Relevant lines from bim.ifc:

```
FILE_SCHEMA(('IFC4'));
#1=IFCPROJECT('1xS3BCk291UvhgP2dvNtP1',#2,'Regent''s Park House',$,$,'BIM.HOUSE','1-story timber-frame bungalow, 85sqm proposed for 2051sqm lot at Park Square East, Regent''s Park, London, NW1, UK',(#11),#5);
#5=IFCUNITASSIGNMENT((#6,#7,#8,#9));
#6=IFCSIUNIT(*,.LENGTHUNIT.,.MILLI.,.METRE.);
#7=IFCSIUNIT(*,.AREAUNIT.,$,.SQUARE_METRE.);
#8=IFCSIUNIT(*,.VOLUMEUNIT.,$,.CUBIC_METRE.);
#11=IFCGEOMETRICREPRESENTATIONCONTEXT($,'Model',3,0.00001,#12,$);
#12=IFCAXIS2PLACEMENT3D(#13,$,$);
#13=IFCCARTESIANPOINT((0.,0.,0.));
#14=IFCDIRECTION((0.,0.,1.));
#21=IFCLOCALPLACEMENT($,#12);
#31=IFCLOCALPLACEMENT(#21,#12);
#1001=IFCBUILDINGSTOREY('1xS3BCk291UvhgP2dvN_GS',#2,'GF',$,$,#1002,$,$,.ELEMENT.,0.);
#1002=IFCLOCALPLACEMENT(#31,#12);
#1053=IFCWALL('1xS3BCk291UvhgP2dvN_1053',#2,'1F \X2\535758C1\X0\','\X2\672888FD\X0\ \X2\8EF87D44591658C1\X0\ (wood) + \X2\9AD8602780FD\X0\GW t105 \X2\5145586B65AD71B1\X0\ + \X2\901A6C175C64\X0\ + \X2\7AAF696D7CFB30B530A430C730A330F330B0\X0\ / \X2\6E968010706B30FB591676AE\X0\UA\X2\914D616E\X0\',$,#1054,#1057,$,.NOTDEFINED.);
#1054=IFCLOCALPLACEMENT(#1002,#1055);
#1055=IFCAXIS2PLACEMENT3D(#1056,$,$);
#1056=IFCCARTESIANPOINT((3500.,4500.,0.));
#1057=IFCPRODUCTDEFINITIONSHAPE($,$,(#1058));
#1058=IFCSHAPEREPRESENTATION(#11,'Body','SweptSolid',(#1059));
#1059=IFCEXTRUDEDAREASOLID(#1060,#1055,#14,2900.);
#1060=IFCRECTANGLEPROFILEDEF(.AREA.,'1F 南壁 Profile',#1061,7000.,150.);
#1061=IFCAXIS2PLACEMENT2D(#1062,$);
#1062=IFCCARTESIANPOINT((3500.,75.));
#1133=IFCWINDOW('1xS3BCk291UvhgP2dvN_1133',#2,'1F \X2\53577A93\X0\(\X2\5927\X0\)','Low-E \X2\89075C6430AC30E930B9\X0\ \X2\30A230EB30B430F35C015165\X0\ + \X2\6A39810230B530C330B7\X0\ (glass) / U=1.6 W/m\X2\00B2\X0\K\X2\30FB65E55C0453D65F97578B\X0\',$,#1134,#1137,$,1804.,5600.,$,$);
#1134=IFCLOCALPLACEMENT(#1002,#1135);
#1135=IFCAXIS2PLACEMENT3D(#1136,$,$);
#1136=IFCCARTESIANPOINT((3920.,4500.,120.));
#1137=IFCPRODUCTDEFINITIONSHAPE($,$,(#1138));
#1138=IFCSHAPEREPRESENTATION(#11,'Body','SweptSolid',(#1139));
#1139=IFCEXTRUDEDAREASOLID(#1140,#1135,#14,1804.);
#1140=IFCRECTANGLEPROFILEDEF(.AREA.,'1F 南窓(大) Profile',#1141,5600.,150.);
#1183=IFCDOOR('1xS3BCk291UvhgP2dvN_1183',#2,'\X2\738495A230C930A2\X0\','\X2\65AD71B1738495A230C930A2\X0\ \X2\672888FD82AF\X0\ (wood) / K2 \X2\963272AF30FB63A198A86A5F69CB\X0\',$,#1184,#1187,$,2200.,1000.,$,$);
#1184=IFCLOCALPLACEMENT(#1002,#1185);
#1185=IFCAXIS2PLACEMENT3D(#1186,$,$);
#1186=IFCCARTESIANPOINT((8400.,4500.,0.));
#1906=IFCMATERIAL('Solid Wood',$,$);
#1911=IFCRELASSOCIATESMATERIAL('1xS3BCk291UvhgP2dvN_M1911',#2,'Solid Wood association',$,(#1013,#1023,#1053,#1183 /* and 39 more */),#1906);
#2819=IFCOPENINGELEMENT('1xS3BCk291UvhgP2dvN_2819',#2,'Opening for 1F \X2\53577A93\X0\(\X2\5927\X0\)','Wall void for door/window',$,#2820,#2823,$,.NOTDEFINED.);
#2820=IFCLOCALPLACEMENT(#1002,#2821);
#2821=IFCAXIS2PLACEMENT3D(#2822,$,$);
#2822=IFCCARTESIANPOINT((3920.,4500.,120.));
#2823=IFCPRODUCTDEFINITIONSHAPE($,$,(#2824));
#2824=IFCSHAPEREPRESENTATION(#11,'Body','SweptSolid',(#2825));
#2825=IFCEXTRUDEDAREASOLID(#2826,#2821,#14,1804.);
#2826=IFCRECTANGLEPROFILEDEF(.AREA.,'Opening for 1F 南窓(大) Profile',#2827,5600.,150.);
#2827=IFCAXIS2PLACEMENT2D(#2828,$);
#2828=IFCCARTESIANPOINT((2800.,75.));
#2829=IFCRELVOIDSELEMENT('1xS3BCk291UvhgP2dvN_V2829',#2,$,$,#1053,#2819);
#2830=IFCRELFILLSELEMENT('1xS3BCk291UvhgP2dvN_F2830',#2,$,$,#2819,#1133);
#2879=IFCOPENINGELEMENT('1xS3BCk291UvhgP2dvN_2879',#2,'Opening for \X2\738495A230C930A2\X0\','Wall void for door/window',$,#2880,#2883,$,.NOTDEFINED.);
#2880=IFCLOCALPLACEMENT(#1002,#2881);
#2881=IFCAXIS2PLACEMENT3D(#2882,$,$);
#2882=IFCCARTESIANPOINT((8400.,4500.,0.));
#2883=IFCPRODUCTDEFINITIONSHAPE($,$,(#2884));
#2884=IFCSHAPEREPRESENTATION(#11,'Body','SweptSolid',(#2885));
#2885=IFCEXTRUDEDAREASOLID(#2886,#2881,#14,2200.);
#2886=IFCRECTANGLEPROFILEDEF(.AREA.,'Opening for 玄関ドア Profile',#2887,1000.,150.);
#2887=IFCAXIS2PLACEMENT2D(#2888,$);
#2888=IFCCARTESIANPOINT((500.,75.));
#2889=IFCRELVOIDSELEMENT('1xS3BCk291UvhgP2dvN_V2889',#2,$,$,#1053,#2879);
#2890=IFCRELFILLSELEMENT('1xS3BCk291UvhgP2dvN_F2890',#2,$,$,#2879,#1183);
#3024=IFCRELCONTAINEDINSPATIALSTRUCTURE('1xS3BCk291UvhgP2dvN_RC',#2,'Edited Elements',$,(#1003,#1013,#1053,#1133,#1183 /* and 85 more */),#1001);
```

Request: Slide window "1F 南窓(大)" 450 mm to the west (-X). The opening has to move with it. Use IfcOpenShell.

```python
import ifcopenshell
import ifcopenshell.api.geometry
import ifcopenshell.util.placement
import ifcopenshell.util.unit

model = ifcopenshell.open("bim.ifc")
unit_scale = ifcopenshell.util.unit.calculate_unit_scale(model)

window = model.by_guid("1xS3BCk291UvhgP2dvN_1133")
opening = window.FillsVoids[0].RelatingOpeningElement
wall = opening.VoidsElements[0].RelatingBuildingElement

wall_matrix = ifcopenshell.util.placement.get_local_placement(wall.ObjectPlacement)
shift = wall_matrix[:3, 0] * -0.45 / unit_scale
before = ifcopenshell.util.placement.get_local_placement(window.ObjectPlacement)[:3, 3].copy()

# The window is not placed relative to its opening, so move both.
for product in (opening, window):
    matrix = ifcopenshell.util.placement.get_local_placement(product.ObjectPlacement)
    matrix[:3, 3] += shift
    ifcopenshell.api.geometry.edit_object_placement(model, product=product, matrix=matrix, is_si=False)

after = ifcopenshell.util.placement.get_local_placement(window.ObjectPlacement)[:3, 3]
print("window moved by", (after - before).round(3) + 0.0)

model.write("bim-out.ifc")
```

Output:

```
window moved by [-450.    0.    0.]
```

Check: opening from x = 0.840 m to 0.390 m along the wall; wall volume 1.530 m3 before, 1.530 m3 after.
